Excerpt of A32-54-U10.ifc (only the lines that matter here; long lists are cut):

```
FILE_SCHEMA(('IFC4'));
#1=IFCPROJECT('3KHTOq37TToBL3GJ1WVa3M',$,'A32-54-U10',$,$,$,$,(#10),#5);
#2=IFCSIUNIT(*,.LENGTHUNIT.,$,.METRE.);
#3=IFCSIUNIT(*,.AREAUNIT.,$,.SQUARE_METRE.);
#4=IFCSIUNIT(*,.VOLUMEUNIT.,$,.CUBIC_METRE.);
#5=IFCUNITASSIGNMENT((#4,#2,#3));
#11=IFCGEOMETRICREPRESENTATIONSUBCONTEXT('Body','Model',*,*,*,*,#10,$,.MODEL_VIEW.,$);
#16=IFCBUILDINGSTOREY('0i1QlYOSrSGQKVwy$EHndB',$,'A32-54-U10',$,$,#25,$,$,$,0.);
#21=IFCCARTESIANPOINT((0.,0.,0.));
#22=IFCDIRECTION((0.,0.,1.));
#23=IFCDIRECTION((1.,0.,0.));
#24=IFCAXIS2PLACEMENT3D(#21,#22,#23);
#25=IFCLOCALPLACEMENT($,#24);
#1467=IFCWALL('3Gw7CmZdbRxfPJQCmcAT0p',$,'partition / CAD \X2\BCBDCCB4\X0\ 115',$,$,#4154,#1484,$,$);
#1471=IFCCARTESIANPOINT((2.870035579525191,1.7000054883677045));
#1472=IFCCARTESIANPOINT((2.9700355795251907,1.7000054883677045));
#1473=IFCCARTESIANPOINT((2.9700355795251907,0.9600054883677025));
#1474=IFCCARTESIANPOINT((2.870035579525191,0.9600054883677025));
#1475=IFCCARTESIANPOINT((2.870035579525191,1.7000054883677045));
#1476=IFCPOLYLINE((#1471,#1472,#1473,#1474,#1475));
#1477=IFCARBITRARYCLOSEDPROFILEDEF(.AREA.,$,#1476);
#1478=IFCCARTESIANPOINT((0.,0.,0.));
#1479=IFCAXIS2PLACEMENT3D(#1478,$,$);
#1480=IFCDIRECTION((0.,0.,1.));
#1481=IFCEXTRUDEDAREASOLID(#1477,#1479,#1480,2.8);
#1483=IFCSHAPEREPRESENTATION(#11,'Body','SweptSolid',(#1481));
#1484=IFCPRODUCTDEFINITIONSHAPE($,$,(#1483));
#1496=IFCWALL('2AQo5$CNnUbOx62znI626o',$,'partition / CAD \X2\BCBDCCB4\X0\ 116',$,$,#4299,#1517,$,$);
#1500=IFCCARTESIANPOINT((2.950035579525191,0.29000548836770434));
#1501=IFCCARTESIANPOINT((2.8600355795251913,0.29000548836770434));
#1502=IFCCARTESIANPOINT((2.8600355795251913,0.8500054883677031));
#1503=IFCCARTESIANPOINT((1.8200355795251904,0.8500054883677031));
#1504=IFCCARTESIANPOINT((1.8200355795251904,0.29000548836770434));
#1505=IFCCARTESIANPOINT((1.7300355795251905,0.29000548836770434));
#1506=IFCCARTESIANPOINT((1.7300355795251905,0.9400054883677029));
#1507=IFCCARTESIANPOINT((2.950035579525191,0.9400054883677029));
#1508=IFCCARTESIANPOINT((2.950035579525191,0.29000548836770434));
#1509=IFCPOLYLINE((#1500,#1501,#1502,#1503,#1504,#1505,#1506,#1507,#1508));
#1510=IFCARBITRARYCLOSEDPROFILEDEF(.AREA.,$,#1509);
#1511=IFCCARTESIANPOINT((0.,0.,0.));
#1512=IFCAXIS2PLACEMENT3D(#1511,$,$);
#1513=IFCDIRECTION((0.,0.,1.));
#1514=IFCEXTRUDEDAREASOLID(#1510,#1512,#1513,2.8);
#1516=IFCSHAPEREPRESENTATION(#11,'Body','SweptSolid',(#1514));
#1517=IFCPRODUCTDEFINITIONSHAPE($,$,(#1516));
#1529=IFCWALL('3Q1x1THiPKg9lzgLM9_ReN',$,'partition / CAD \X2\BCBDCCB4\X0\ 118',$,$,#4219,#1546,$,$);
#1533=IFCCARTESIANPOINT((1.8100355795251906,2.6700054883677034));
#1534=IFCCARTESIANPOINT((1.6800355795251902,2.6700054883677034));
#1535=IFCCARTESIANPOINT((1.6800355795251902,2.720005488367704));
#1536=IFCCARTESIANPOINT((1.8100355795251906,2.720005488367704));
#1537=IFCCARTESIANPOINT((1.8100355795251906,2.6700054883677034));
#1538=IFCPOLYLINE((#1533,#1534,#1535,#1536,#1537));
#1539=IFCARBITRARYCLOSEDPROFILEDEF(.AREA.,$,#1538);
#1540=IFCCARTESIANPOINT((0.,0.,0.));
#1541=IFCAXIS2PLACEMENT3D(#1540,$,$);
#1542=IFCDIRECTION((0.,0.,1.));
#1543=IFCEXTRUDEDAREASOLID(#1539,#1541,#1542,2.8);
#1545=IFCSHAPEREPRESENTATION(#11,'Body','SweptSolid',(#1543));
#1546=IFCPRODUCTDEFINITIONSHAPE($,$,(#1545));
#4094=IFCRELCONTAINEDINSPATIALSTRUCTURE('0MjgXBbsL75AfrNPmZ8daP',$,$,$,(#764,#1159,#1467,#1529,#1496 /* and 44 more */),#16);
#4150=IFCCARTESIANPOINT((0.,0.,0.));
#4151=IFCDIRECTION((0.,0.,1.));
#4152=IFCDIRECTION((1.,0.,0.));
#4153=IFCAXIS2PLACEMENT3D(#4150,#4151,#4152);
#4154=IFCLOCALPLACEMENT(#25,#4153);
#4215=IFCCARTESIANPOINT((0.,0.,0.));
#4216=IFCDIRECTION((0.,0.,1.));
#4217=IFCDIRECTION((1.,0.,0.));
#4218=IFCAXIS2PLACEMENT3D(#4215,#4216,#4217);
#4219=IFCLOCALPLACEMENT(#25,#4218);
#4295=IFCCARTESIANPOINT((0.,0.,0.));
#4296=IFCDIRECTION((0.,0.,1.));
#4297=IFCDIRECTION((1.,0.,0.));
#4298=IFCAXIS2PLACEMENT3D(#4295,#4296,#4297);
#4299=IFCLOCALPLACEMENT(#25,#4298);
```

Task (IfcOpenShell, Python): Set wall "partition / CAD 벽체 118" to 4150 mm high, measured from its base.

```python
import ifcopenshell
import ifcopenshell.geom
import ifcopenshell.util.representation
import ifcopenshell.util.shape

model = ifcopenshell.open("A32-54-U10.ifc")
settings = ifcopenshell.geom.settings()


def volume(element):
    """Net volume in cubic metres, openings subtracted."""
    shape = ifcopenshell.geom.create_shape(settings, element)
    return ifcopenshell.util.shape.get_volume(shape.geometry)


wall = model.by_guid("3Q1x1THiPKg9lzgLM9_ReN")
before = volume(wall)

body = ifcopenshell.util.representation.get_representation(wall, "Model", "Body")
solid = body.Items[0]
old_height = solid.Depth
solid.Depth = 4.15
after = volume(wall)

print(f"height {old_height:g} -> {solid.Depth:g}, volume {before:.3f} -> {after:.3f} m3")

model.write("A32-54-U10_edited.ifc")
```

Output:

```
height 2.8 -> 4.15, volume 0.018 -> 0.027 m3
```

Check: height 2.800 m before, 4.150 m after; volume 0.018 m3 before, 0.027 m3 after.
